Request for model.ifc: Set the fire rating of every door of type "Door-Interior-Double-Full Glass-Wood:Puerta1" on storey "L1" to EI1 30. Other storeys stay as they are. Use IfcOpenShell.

First a look at what the model holds.

```python
import ifcopenshell
import ifcopenshell.util.element

model = ifcopenshell.open("model.ifc")
print(model.schema)
storey = next(s for s in model.by_type("IfcBuildingStorey") if s.Name == "L1")
doors = [e for e in ifcopenshell.util.element.get_decomposition(storey) if e.is_a("IfcDoor")]
seen = {}
for e in doors:
    element_type = ifcopenshell.util.element.get_type(e)
    key = (element_type.Name if element_type != e and element_type else None, ifcopenshell.util.element.get_pset(e, "Pset_DoorCommon", "FireRating"))
    seen[key] = seen.get(key, 0) + 1
for (name, value), count in sorted(seen.items(), key=str):
    print(count, "x", name, "|", value)
```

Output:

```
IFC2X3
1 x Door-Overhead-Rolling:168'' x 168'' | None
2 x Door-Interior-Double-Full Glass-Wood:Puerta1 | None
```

```python
import ifcopenshell
import ifcopenshell.api.pset
import ifcopenshell.util.element

model = ifcopenshell.open("model.ifc")

storey = next(s for s in model.by_type("IfcBuildingStorey") if s.Name == "L1")
doors = [e for e in ifcopenshell.util.element.get_decomposition(storey) if e.is_a("IfcDoor")]

count = 0
for e in doors:
    element_type = ifcopenshell.util.element.get_type(e)
    if element_type in (None, e) or element_type.Name != "Door-Interior-Double-Full Glass-Wood:Puerta1":
        continue
    # add_pset returns the element's existing set when there is one.
    pset = ifcopenshell.api.pset.add_pset(model, product=e, name="Pset_DoorCommon")
    ifcopenshell.api.pset.edit_pset(model, pset=pset, properties={"FireRating": "EI1 30"})
    count += 1

print(count, "doors updated")

model.write("model_edited.ifc")
```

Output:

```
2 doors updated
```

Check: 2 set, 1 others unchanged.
